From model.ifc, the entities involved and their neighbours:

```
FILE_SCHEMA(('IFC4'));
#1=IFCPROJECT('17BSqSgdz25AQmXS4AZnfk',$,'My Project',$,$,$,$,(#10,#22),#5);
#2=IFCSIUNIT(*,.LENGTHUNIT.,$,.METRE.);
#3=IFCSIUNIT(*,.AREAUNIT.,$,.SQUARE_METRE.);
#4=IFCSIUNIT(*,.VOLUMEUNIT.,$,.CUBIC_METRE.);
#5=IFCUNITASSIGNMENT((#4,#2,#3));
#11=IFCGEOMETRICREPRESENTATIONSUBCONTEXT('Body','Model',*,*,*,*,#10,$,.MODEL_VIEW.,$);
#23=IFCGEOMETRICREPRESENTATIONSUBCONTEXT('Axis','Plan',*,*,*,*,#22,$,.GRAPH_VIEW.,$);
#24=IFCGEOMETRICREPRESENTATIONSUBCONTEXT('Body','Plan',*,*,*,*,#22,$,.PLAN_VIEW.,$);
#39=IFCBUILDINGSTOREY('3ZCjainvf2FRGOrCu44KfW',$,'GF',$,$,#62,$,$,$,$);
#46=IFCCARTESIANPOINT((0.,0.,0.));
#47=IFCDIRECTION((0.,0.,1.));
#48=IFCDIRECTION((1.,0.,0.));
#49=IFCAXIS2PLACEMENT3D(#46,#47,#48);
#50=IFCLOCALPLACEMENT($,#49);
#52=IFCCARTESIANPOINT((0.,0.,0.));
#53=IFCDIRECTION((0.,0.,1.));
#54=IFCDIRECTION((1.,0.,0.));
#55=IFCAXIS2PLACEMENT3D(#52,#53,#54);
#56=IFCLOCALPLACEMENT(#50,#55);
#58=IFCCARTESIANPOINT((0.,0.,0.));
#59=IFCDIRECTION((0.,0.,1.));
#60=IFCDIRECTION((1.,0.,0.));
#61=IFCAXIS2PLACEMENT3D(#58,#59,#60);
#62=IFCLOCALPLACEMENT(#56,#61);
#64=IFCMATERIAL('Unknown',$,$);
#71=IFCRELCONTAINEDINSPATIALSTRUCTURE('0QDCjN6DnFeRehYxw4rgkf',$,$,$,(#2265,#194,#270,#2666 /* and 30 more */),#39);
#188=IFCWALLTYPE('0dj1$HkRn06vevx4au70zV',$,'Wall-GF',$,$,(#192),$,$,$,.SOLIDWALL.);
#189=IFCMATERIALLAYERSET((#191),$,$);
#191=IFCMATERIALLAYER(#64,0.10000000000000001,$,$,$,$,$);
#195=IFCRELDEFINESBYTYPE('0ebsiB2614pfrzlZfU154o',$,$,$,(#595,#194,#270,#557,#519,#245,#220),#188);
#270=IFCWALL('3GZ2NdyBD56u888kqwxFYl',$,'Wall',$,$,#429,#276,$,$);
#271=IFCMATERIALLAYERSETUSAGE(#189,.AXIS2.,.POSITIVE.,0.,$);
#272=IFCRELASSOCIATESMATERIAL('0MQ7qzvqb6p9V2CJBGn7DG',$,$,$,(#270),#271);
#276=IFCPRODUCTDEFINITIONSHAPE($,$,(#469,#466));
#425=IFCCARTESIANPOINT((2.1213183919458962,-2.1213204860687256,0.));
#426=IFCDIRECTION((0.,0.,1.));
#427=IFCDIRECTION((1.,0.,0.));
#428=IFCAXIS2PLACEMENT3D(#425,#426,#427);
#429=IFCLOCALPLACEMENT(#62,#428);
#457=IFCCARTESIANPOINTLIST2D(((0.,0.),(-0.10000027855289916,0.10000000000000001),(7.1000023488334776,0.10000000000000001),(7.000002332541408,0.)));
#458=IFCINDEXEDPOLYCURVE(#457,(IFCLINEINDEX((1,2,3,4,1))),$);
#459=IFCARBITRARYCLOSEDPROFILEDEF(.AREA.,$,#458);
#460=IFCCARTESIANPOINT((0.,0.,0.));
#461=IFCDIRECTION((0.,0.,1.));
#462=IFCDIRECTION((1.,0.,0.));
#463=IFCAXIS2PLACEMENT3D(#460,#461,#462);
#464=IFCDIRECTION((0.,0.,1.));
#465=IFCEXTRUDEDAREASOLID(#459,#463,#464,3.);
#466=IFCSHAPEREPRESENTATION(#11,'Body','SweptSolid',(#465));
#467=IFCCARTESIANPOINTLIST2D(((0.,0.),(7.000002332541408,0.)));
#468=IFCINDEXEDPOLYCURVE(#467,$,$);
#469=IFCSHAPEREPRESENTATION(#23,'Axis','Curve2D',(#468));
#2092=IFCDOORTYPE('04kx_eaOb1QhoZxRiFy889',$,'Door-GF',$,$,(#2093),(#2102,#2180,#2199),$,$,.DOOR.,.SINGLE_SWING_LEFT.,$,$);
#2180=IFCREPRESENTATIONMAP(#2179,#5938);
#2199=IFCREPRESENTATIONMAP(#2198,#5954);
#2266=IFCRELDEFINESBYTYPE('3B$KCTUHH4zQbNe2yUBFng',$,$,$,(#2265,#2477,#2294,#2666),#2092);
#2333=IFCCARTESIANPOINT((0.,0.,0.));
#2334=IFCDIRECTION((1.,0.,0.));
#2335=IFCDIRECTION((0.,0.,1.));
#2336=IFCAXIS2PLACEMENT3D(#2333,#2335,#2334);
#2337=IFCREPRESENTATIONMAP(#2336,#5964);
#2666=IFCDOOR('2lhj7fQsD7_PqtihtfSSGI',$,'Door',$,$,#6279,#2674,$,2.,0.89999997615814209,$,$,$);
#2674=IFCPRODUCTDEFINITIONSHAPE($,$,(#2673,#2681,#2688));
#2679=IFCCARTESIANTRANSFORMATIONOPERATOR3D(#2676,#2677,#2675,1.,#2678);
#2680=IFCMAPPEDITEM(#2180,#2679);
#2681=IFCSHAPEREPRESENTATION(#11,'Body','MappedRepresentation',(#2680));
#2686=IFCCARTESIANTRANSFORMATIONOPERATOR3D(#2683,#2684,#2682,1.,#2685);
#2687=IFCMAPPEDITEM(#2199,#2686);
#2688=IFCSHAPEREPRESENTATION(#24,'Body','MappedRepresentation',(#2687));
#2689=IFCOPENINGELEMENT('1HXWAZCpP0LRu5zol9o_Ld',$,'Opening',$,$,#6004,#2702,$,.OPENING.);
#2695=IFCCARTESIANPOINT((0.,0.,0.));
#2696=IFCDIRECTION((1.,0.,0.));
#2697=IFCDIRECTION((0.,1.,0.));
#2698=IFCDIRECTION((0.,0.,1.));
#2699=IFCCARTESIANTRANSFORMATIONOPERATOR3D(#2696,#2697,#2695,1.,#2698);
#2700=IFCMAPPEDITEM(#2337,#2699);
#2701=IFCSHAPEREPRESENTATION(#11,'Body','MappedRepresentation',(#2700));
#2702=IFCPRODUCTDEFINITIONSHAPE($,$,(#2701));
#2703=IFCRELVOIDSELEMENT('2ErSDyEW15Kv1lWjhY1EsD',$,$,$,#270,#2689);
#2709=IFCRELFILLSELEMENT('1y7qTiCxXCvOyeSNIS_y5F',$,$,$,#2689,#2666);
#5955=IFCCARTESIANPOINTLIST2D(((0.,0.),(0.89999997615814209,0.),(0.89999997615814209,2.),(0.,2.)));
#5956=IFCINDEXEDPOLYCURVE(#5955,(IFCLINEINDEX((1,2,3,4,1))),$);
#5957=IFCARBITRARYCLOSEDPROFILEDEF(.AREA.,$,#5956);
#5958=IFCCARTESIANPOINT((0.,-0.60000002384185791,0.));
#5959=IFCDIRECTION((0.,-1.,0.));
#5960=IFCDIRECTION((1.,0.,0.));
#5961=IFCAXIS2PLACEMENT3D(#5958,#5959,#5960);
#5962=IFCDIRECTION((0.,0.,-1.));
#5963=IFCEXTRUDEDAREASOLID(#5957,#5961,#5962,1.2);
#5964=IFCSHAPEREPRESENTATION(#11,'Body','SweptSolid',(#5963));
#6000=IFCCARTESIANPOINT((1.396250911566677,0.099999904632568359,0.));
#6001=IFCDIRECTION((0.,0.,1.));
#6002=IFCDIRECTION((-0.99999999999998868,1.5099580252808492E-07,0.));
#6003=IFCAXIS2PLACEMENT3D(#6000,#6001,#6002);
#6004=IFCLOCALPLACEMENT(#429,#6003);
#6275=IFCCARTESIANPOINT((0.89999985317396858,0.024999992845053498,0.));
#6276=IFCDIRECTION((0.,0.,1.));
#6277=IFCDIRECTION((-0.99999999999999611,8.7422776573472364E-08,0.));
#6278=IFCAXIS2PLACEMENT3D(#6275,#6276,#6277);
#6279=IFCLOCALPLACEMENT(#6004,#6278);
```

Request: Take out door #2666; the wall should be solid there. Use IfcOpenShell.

```python
import ifcopenshell
import ifcopenshell.api.feature
import ifcopenshell.api.root
import ifcopenshell.geom
import ifcopenshell.util.shape

model = ifcopenshell.open("model.ifc")
settings = ifcopenshell.geom.settings()


def volume(element):
    """Net volume in cubic metres, openings subtracted."""
    shape = ifcopenshell.geom.create_shape(settings, element)
    return ifcopenshell.util.shape.get_volume(shape.geometry)


door = model.by_guid("2lhj7fQsD7_PqtihtfSSGI")
opening = door.FillsVoids[0].RelatingOpeningElement
wall = opening.VoidsElements[0].RelatingBuildingElement
before = volume(wall)

ifcopenshell.api.root.remove_product(model, product=door)
ifcopenshell.api.feature.remove_feature(model, feature=opening)

after = volume(wall)

print(f"wall volume {before:.3f} -> {after:.3f} m3")

model.write("model_rev.ifc")
```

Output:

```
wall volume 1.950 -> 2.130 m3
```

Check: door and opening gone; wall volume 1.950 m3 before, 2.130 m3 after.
